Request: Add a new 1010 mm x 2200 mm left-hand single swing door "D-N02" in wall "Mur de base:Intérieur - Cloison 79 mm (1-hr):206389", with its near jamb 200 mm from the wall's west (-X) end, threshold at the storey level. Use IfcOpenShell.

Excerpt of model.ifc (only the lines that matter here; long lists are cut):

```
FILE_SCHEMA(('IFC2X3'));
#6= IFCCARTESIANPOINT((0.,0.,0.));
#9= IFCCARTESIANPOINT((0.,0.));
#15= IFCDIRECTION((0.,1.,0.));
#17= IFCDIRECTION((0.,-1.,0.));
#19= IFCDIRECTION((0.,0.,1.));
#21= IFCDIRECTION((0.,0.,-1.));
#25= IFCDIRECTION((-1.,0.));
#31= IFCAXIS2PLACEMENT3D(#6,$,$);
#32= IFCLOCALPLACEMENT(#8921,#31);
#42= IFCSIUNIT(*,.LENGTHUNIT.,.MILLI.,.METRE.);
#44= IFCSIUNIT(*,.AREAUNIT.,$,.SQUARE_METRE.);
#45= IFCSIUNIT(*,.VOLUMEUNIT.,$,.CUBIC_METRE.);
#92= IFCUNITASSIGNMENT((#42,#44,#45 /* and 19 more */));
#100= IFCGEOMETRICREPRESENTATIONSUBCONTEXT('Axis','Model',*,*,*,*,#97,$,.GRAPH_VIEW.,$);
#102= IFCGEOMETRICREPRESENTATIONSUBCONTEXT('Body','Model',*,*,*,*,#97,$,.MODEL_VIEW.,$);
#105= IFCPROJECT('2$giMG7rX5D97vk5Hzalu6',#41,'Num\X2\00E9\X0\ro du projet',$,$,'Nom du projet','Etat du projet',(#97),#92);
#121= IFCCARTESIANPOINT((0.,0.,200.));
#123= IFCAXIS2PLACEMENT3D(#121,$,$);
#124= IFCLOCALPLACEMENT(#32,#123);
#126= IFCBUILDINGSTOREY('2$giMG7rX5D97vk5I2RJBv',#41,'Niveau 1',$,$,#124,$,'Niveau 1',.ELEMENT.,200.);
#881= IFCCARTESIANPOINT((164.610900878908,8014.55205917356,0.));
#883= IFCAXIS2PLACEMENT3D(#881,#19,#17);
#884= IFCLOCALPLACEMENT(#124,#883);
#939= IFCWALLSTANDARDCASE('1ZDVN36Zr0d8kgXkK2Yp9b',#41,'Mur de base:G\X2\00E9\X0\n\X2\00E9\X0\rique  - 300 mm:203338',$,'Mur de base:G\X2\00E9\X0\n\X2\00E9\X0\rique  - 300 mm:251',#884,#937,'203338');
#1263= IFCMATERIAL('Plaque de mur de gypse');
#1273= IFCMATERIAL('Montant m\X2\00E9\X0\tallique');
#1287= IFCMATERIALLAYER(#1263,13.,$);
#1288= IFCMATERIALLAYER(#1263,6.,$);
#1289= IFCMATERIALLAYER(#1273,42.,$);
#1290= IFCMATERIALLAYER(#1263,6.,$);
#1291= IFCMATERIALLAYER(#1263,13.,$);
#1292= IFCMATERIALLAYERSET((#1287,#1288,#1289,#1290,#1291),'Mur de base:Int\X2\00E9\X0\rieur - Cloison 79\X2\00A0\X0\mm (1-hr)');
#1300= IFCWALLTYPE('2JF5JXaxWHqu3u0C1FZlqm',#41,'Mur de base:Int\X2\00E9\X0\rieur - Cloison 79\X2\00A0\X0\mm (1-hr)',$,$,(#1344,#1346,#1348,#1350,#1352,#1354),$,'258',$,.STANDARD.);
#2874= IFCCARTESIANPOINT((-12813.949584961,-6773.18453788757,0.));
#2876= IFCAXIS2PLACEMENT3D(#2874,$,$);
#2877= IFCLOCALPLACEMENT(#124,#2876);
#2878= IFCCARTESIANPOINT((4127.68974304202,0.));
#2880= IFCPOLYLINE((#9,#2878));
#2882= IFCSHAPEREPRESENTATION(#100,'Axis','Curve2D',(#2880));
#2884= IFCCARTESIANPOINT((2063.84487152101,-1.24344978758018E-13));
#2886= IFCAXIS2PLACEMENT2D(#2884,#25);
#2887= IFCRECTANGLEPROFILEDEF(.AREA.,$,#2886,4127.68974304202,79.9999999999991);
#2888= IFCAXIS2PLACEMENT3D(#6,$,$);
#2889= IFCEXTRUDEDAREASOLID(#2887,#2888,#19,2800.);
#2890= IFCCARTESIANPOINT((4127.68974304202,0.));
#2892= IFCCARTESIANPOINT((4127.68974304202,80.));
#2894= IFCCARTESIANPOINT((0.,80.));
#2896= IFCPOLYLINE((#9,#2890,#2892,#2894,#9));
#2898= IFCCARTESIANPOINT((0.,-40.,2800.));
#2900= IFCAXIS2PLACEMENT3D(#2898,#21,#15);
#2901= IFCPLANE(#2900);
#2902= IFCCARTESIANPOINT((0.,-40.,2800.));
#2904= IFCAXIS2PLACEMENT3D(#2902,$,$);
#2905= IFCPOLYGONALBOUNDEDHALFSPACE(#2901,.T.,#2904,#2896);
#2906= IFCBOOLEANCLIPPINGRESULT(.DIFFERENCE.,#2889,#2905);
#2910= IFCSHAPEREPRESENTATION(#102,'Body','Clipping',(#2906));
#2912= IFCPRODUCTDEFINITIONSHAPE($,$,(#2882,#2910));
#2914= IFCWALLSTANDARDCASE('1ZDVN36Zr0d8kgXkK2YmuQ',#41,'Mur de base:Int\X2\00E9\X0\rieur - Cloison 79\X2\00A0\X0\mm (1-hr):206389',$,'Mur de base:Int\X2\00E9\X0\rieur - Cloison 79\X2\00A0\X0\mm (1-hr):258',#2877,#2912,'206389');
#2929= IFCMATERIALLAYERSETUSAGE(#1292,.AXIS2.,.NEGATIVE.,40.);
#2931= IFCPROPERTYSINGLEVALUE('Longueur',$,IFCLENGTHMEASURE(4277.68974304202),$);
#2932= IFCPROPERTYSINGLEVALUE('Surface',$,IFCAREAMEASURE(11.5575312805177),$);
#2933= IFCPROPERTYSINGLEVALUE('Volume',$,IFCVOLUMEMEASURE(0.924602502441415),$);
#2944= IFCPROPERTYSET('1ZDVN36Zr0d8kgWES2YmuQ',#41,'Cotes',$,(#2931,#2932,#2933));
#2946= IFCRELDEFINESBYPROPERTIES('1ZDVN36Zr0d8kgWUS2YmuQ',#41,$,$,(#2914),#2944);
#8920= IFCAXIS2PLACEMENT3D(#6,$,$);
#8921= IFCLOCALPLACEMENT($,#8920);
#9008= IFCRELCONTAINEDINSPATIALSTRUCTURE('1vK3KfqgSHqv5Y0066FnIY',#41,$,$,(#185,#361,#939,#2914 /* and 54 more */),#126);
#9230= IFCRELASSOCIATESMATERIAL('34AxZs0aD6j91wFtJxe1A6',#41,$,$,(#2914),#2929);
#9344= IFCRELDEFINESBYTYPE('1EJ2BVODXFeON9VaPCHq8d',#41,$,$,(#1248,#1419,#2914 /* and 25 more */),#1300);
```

```python
import numpy as np
import ifcopenshell
import ifcopenshell.api.feature
import ifcopenshell.api.geometry
import ifcopenshell.api.pset
import ifcopenshell.api.root
import ifcopenshell.api.spatial
import ifcopenshell.api.type
import ifcopenshell.geom
import ifcopenshell.util.element
import ifcopenshell.util.placement
import ifcopenshell.util.representation
import ifcopenshell.util.shape
import ifcopenshell.util.unit

model = ifcopenshell.open("model.ifc")
unit_scale = ifcopenshell.util.unit.calculate_unit_scale(model)
area_scale = ifcopenshell.util.unit.calculate_unit_scale(model, "AREAUNIT")
volume_scale = ifcopenshell.util.unit.calculate_unit_scale(model, "VOLUMEUNIT")
settings = ifcopenshell.geom.settings()


def volume(element):
    """Net volume in cubic metres, openings subtracted."""
    shape = ifcopenshell.geom.create_shape(settings, element)
    return ifcopenshell.util.shape.get_volume(shape.geometry)


wall = model.by_id(2914)
storey = ifcopenshell.util.element.get_container(wall, ifc_class="IfcBuildingStorey")
context = ifcopenshell.util.representation.get_context(model, "Model", "Body", "MODEL_VIEW")
before = volume(wall)

width, height, from_end, sill = 1.01, 2.2, 0.2, 0.0  # metres

# The wall runs along its own X axis, and the end named is its -X end.
wall_shape = ifcopenshell.geom.create_shape(settings, wall)
x, y, z = ifcopenshell.util.shape.get_vertices(wall_shape.geometry).T
start = x.min() + from_end
face, thickness = float(y.min()), float(y.max() - y.min())
wall_matrix = ifcopenshell.util.placement.get_local_placement(wall.ObjectPlacement)
level = ifcopenshell.util.placement.get_local_placement(storey.ObjectPlacement)[2, 3]


def in_wall(x, y):
    """Placement at x, y metres in the wall's axes, at sill height."""
    matrix = wall_matrix.copy()
    matrix[:, 3] = wall_matrix @ np.array([x / unit_scale, y / unit_scale, 0.0, 1.0])
    matrix[2, 3] = level + sill / unit_scale
    return matrix


# Opening: a box that overshoots both wall faces by 50 mm.
opening = ifcopenshell.api.root.create_entity(model, ifc_class="IfcOpeningElement")
box = ifcopenshell.api.geometry.add_wall_representation(
    model, context=context, length=width, height=height, thickness=thickness + 0.1
)
ifcopenshell.api.geometry.assign_representation(model, product=opening, representation=box)
ifcopenshell.api.geometry.edit_object_placement(model, product=opening, matrix=in_wall(start, face - 0.05), is_si=False)
ifcopenshell.api.feature.add_feature(model, feature=opening, element=wall)

door = ifcopenshell.api.root.create_entity(model, ifc_class="IfcDoor", name="D-N02")
door.OverallWidth, door.OverallHeight = width / unit_scale, height / unit_scale
body = ifcopenshell.api.geometry.add_door_representation(
    model,
    context=context,
    overall_width=door.OverallWidth,
    overall_height=door.OverallHeight,
    operation_type="SINGLE_SWING_LEFT",
    lining_properties={"LiningDepth": thickness / unit_scale, "ThresholdDepth": thickness / unit_scale},
)
ifcopenshell.api.geometry.assign_representation(model, product=door, representation=body)
ifcopenshell.api.spatial.assign_container(model, products=[door], relating_structure=storey)
fills = ifcopenshell.api.feature.add_filling(model, opening=opening, element=door)
fills.OwnerHistory = door.OwnerHistory  # required in IFC2X3

# IFC2X3 keeps the operation on the door style.
style = ifcopenshell.api.root.create_entity(model, ifc_class="IfcDoorStyle", name="D-N02")
style.OperationType, style.ConstructionType = "SINGLE_SWING_LEFT", "NOTDEFINED"
style.ParameterTakesPrecedence = style.Sizeable = False
ifcopenshell.api.type.assign_type(model, related_objects=[door], relating_type=style)

# The lining spans the wall, so the door starts at the wall face.
ifcopenshell.api.geometry.edit_object_placement(model, product=door, matrix=in_wall(start, face), is_si=False)

after = volume(wall)

# Update the wall's stored quantities.
pset = model.by_id(ifcopenshell.util.element.get_pset(wall, "Cotes", should_inherit=False)["id"])
ifcopenshell.api.pset.edit_pset(model, pset=pset, properties={
    "Surface": model.create_entity("IfcAreaMeasure", after / thickness / area_scale),
    "Volume": model.create_entity("IfcVolumeMeasure", after / volume_scale),
})

print(f"wall volume {before:.3f} -> {after:.3f} m3")

model.write("model_rev.ifc")
```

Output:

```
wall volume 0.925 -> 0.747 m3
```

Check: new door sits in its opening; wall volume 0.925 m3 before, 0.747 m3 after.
